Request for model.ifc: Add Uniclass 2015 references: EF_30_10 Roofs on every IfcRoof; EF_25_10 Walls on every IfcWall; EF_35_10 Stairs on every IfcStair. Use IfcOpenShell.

First a look at what the model holds.

```python
import ifcopenshell

model = ifcopenshell.open("model.ifc")
print(model.schema)
print("classifications:", [c.Name for c in model.by_type("IfcClassification")])
for ifc_class in ("IfcDoor", "IfcRoof", "IfcStair", "IfcWall", "IfcWindow"):
    print(ifc_class, len(model.by_type(ifc_class)))
```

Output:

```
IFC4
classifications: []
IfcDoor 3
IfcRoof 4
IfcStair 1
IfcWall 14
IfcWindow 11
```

```python
import ifcopenshell
import ifcopenshell.api.classification

model = ifcopenshell.open("model.ifc")

system = ifcopenshell.api.classification.add_classification(model, classification="Uniclass 2015")

codes = {
    "IfcRoof": ("EF_30_10", "Roofs"),
    "IfcWall": ("EF_25_10", "Walls"),
    "IfcStair": ("EF_35_10", "Stairs"),
}
for ifc_class, (code, name) in codes.items():
    products = model.by_type(ifc_class)
    ifcopenshell.api.classification.add_reference(
        model, products=products, classification=system, identification=code, name=name
    )
    print(code, len(products))

model.write("model_v2.ifc")
```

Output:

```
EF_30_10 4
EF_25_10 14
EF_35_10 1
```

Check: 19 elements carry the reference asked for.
